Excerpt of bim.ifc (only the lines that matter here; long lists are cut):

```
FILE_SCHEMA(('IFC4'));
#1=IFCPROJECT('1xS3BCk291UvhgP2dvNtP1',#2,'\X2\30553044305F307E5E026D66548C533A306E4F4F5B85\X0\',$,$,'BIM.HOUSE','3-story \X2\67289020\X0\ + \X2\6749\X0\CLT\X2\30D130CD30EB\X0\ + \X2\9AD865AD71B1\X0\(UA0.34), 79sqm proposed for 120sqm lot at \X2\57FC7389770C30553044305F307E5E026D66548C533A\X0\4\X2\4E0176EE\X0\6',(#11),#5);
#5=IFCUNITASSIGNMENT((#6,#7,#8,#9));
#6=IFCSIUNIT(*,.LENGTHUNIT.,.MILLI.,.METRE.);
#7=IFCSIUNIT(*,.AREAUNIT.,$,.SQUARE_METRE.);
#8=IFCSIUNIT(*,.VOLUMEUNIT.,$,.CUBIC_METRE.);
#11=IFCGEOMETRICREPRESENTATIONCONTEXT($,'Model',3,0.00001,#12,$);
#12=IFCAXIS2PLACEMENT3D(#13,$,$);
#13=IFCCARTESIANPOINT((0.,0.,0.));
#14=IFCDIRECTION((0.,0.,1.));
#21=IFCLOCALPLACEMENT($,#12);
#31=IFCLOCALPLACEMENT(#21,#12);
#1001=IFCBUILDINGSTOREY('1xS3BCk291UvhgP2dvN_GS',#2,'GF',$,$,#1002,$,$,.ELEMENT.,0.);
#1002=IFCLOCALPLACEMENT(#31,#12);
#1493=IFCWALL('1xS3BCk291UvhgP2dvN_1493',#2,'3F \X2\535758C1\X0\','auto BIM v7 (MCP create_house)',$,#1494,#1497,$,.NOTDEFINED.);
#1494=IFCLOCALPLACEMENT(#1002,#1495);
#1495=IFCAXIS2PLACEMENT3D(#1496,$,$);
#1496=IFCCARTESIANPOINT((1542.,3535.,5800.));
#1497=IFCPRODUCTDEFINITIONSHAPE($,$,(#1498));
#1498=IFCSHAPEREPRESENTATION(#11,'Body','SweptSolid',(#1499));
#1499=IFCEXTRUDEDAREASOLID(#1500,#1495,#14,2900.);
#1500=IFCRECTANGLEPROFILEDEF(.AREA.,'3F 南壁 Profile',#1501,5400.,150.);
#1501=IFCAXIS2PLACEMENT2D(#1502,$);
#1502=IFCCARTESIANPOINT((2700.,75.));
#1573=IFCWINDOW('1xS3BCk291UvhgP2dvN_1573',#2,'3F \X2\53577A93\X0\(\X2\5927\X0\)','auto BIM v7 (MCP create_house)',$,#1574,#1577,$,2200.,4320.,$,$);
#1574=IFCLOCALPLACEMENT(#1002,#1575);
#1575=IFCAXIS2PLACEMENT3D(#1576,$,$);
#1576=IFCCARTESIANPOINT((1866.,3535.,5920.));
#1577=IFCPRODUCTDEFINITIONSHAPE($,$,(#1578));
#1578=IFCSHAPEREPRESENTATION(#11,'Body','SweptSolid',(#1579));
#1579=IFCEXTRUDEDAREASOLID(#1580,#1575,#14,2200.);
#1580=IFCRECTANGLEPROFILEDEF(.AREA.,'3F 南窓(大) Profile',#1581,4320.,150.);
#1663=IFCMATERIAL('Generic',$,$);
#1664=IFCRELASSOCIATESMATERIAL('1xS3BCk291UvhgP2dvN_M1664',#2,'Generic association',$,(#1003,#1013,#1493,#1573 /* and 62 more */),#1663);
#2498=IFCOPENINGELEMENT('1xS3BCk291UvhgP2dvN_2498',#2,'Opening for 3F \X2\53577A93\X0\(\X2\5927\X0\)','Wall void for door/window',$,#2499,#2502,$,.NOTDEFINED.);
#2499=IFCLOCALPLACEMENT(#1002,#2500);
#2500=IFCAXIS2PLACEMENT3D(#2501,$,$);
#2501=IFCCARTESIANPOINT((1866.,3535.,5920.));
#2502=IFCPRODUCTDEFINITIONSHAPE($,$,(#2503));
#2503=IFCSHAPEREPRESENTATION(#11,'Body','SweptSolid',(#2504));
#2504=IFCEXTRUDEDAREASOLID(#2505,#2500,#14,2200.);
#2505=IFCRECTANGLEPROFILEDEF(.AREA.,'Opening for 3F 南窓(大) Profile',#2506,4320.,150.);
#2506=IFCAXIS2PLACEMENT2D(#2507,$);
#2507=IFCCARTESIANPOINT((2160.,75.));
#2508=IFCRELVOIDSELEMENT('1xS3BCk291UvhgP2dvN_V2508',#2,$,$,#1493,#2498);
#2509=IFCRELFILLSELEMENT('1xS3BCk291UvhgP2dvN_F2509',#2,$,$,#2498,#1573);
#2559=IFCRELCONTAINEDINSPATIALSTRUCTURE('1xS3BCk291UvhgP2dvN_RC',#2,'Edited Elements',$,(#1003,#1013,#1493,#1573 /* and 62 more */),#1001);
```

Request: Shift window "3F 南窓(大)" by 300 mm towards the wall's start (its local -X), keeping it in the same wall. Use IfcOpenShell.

```python
import ifcopenshell
import ifcopenshell.api.geometry
import ifcopenshell.util.placement

model = ifcopenshell.open("bim.ifc")

window = model.by_guid("1xS3BCk291UvhgP2dvN_1573")
opening = window.FillsVoids[0].RelatingOpeningElement
wall = opening.VoidsElements[0].RelatingBuildingElement

wall_matrix = ifcopenshell.util.placement.get_local_placement(wall.ObjectPlacement)
shift = wall_matrix[:3, 0] * -300.0
before = ifcopenshell.util.placement.get_local_placement(window.ObjectPlacement)[:3, 3].copy()

# The window is not placed relative to its opening, so move both.
for product in (opening, window):
    matrix = ifcopenshell.util.placement.get_local_placement(product.ObjectPlacement)
    matrix[:3, 3] += shift
    ifcopenshell.api.geometry.edit_object_placement(model, product=product, matrix=matrix, is_si=False)

after = ifcopenshell.util.placement.get_local_placement(window.ObjectPlacement)[:3, 3]
print("window moved by", (after - before).round(3) + 0.0)

model.write("bim_edited.ifc")
```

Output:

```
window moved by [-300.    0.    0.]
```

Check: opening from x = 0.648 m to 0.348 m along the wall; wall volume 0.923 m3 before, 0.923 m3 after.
